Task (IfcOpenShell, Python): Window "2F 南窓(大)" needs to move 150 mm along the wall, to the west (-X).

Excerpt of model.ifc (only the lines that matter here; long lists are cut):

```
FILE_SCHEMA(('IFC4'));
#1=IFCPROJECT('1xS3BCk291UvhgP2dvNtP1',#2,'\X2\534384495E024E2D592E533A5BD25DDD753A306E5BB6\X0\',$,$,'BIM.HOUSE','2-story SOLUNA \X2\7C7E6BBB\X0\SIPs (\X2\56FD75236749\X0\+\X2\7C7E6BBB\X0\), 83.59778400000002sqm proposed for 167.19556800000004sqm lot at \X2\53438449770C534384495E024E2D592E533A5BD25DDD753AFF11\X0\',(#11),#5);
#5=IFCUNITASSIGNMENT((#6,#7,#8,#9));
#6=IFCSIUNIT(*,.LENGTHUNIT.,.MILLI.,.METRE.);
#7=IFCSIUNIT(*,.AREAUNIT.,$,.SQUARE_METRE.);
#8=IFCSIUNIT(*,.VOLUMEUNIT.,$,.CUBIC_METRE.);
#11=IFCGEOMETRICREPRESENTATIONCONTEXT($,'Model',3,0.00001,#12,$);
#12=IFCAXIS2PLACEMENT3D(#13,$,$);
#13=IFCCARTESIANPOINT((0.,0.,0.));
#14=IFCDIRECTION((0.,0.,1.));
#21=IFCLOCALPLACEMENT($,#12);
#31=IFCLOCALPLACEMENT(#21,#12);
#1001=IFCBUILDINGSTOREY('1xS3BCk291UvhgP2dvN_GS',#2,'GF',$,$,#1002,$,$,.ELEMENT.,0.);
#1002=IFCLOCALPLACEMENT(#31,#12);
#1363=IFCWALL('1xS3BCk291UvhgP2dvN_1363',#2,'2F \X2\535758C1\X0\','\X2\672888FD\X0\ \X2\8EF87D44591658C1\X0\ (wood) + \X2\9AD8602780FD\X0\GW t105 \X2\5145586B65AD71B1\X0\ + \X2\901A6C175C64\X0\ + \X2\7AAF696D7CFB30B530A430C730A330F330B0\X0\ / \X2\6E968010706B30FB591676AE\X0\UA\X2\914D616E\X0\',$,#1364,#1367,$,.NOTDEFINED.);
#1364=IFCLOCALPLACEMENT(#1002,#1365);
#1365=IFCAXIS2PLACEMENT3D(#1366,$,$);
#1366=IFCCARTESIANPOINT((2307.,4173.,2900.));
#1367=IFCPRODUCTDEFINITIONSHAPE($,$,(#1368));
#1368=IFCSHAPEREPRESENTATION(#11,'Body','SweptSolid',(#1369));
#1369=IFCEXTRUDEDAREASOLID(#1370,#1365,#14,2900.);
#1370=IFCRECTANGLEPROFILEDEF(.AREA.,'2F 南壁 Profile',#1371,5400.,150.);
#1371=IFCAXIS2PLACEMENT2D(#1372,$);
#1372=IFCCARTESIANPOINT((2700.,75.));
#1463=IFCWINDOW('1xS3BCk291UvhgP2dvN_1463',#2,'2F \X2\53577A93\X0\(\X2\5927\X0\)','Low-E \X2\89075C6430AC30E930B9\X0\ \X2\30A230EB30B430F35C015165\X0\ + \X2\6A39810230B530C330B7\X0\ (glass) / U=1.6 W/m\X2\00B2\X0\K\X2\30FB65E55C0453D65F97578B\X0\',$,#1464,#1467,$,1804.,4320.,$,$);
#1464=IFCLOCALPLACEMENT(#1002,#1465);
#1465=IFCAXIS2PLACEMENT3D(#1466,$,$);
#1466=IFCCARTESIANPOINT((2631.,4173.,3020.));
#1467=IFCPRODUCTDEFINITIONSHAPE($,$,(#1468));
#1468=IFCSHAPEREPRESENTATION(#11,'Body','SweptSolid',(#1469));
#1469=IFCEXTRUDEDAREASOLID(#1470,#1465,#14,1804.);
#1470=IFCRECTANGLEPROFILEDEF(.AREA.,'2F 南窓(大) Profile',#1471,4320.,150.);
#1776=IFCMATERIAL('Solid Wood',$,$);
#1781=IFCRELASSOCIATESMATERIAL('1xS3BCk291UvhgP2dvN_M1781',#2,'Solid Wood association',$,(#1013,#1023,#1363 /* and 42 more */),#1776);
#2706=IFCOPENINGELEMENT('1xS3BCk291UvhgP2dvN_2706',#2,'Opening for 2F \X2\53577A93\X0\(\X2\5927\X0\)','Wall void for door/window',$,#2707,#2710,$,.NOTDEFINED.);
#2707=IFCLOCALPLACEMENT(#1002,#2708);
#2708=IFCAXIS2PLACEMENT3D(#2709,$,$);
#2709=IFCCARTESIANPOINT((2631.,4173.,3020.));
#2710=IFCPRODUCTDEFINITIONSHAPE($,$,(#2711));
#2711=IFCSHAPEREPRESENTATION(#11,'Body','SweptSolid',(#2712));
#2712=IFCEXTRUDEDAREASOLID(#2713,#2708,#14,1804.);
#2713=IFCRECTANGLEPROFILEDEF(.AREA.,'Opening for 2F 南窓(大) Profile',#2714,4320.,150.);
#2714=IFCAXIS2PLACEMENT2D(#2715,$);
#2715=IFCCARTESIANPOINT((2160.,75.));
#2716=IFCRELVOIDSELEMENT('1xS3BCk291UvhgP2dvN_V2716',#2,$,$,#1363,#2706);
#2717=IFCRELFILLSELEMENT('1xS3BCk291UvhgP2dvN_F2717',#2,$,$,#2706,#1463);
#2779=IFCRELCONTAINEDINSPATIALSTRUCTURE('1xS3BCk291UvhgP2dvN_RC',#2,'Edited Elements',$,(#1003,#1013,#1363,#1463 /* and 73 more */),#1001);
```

```python
import ifcopenshell
import ifcopenshell.api.geometry
import ifcopenshell.util.placement
import ifcopenshell.util.unit

model = ifcopenshell.open("model.ifc")
unit_scale = ifcopenshell.util.unit.calculate_unit_scale(model)

window = model.by_guid("1xS3BCk291UvhgP2dvN_1463")
opening = window.FillsVoids[0].RelatingOpeningElement
wall = opening.VoidsElements[0].RelatingBuildingElement

wall_matrix = ifcopenshell.util.placement.get_local_placement(wall.ObjectPlacement)
shift = wall_matrix[:3, 0] * -0.15 / unit_scale
before = ifcopenshell.util.placement.get_local_placement(window.ObjectPlacement)[:3, 3].copy()

# The window is not placed relative to its opening, so move both.
for product in (opening, window):
    matrix = ifcopenshell.util.placement.get_local_placement(product.ObjectPlacement)
    matrix[:3, 3] += shift
    ifcopenshell.api.geometry.edit_object_placement(model, product=product, matrix=matrix, is_si=False)

after = ifcopenshell.util.placement.get_local_placement(window.ObjectPlacement)[:3, 3]
print("window moved by", (after - before).round(3) + 0.0)

model.write("model_rev.ifc")
```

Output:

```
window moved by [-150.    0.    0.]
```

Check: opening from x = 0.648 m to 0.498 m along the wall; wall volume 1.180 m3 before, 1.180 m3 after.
